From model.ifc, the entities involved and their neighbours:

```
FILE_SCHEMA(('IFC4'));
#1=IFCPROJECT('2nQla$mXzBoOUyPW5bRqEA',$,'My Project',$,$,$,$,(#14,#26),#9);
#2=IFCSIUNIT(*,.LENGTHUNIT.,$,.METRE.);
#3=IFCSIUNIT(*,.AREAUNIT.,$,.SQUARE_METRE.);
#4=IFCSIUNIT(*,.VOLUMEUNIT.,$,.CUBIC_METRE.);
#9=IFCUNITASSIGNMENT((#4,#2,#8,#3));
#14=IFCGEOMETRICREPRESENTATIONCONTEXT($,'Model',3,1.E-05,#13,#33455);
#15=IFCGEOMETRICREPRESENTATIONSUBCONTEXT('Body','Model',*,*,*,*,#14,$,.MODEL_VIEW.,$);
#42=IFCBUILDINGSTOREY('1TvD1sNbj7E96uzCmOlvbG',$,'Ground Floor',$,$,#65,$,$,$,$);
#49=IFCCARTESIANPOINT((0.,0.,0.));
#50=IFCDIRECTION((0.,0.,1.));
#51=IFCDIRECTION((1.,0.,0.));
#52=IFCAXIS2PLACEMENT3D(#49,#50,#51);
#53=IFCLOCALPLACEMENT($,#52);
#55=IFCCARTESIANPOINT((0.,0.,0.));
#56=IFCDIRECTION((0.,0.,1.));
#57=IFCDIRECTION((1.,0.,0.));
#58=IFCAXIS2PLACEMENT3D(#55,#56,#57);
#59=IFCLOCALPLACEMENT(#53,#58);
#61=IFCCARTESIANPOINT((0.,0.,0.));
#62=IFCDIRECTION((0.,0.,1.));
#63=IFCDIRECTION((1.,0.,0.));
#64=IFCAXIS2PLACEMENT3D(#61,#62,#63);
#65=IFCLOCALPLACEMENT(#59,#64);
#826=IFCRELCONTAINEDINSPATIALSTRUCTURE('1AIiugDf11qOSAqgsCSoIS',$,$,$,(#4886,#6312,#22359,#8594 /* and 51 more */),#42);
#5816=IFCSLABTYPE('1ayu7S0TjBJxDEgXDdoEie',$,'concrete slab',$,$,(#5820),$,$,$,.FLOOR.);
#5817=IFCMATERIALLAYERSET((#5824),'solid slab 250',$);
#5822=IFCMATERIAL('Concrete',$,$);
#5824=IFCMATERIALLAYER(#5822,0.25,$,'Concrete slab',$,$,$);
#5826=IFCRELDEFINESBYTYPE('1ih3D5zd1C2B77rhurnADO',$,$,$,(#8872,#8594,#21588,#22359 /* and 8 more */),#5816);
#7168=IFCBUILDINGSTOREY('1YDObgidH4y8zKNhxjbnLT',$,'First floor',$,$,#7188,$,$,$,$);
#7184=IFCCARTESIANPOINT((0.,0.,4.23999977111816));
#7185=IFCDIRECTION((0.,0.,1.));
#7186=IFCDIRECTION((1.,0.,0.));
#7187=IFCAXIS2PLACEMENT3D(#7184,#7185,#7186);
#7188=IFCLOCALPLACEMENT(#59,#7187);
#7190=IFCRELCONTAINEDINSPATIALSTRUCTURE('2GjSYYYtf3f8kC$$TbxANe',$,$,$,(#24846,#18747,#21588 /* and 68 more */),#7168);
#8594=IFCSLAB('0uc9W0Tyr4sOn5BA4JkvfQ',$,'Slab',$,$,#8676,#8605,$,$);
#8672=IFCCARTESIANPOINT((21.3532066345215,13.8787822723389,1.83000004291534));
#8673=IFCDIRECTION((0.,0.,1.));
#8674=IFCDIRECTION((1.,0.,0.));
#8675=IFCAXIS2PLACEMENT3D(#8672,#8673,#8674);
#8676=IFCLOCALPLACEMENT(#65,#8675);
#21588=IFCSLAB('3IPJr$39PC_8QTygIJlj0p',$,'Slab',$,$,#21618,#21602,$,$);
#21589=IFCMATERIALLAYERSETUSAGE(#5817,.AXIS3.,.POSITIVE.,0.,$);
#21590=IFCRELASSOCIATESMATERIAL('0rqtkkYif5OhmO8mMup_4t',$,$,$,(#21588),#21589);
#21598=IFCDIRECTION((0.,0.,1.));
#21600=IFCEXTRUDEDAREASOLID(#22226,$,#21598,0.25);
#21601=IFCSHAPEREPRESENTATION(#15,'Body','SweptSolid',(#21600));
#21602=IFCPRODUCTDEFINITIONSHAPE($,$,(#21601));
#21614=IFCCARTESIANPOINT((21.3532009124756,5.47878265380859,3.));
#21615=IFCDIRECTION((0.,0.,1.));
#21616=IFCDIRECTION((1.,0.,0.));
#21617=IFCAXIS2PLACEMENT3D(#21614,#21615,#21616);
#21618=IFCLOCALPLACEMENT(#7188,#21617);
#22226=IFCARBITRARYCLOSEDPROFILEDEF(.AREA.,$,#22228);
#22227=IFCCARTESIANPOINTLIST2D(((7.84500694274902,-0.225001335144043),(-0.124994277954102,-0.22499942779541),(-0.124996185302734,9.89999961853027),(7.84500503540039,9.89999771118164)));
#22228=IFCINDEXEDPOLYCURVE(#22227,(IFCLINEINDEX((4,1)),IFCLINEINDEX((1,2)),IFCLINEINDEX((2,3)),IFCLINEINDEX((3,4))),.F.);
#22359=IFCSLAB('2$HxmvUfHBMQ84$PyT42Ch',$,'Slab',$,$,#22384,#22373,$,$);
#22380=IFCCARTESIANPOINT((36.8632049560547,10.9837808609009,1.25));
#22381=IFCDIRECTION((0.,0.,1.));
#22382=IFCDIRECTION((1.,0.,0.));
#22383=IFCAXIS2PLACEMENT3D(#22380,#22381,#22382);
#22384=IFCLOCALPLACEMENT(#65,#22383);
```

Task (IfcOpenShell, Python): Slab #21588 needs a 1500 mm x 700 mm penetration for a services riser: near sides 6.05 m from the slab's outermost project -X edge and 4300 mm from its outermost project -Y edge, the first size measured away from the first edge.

```python
import numpy as np
import ifcopenshell
import ifcopenshell.api.feature
import ifcopenshell.api.geometry
import ifcopenshell.api.root
import ifcopenshell.geom
import ifcopenshell.util.placement
import ifcopenshell.util.representation
import ifcopenshell.util.shape
import ifcopenshell.util.unit

model = ifcopenshell.open("model.ifc")
unit_scale = ifcopenshell.util.unit.calculate_unit_scale(model)
settings = ifcopenshell.geom.settings()


def volume(element):
    """Net volume in cubic metres, openings subtracted."""
    shape = ifcopenshell.geom.create_shape(settings, element)
    return ifcopenshell.util.shape.get_volume(shape.geometry)


slab = model.by_guid("3IPJr$39PC_8QTygIJlj0p")
before = volume(slab)

# Extent in the slab's own axes, in metres. The edges named are its -X and -Y sides.
slab_shape = ifcopenshell.geom.create_shape(settings, slab)
vertices = ifcopenshell.util.shape.get_vertices(slab_shape.geometry)
x_min, y_min, bottom = vertices.min(axis=0)
top = vertices[:, 2].max()

opening = ifcopenshell.api.root.create_entity(model, ifc_class="IfcOpeningElement", name="Services riser opening", predefined_type="OPENING")
context = ifcopenshell.util.representation.get_context(model, "Model", "Body", "MODEL_VIEW")
width, depth = 1.5, 0.7
outline = [(0.0, 0.0), (width, 0.0), (width, depth), (0.0, depth), (0.0, 0.0)]
# Overshoot both faces by 50 mm so the cut is clean.
shape = ifcopenshell.api.geometry.add_slab_representation(
    model, context=context, depth=top - bottom + 0.1, polyline=outline
)
ifcopenshell.api.geometry.assign_representation(model, product=opening, representation=shape)

matrix = ifcopenshell.util.placement.get_local_placement(slab.ObjectPlacement)
matrix[:, 3] = matrix @ np.append(np.array([x_min + 6.05, y_min + 4.3, bottom - 0.05]) / unit_scale, 1.0)
ifcopenshell.api.geometry.edit_object_placement(model, product=opening, matrix=matrix, is_si=False)
ifcopenshell.api.feature.add_feature(model, feature=opening, element=slab)

after = volume(slab)

print(f"slab volume {before:.3f} -> {after:.3f} m3")

model.write("model_rev.ifc")
```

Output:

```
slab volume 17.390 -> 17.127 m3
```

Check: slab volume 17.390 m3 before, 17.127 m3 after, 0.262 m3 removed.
